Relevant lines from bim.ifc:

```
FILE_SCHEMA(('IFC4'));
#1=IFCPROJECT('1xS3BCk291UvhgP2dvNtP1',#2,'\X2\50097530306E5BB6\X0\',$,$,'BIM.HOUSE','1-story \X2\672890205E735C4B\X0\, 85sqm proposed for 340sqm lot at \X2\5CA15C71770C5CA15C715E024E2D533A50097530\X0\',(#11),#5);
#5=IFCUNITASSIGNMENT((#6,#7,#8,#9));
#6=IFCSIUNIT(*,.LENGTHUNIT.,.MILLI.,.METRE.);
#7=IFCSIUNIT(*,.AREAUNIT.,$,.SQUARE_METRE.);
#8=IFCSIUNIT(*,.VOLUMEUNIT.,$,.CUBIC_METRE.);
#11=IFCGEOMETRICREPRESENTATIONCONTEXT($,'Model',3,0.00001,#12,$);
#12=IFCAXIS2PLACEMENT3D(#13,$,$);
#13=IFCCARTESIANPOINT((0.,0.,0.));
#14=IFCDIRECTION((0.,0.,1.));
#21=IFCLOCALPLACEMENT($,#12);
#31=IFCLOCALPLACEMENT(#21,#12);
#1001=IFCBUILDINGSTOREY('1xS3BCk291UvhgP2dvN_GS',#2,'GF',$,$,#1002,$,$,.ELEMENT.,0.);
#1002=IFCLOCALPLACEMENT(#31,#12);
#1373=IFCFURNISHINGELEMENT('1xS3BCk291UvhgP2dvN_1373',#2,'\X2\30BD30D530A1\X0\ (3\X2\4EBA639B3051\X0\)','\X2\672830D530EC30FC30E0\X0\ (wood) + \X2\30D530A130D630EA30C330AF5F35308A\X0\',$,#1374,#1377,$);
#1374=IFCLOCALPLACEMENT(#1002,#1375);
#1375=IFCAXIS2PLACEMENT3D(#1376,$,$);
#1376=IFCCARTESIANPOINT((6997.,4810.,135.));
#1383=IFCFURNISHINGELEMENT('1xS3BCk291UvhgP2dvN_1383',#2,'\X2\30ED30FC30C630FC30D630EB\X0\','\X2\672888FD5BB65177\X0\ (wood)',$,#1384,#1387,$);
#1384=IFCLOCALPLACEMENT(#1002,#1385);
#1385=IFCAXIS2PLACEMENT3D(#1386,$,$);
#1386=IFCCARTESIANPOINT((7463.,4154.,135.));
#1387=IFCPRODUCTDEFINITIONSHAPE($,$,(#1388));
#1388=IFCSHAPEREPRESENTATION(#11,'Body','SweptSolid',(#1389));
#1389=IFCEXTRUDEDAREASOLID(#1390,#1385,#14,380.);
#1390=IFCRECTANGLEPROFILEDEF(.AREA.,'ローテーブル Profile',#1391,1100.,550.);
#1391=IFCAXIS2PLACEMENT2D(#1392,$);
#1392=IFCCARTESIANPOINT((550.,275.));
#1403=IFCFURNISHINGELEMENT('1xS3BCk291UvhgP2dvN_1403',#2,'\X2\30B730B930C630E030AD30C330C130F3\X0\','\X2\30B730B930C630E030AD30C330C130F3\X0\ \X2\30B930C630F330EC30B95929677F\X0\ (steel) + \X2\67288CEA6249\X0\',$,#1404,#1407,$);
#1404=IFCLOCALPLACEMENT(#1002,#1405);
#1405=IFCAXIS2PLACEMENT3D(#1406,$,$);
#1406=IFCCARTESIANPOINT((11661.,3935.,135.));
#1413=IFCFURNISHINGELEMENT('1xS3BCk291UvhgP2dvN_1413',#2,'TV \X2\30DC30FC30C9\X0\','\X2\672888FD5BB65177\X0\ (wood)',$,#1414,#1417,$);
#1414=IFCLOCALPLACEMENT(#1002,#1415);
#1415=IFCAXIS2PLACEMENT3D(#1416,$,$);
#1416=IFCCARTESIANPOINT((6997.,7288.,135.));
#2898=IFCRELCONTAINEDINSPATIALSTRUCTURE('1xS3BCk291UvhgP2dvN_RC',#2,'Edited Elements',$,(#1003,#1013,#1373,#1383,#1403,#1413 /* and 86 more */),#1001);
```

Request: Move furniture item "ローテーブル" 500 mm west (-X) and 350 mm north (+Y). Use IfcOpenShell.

```python
import ifcopenshell
import ifcopenshell.api.geometry
import ifcopenshell.util.placement
import ifcopenshell.util.unit

model = ifcopenshell.open("bim.ifc")
unit_scale = ifcopenshell.util.unit.calculate_unit_scale(model)

item = model.by_id(1383)
matrix = ifcopenshell.util.placement.get_local_placement(item.ObjectPlacement)
matrix[0, 3] -= 0.5 / unit_scale
matrix[1, 3] += 0.35 / unit_scale
ifcopenshell.api.geometry.edit_object_placement(model, product=item, matrix=matrix, is_si=False)

print(ifcopenshell.util.placement.get_local_placement(item.ObjectPlacement).round(3) + 0.0)

model.write("bim_v2.ifc")
```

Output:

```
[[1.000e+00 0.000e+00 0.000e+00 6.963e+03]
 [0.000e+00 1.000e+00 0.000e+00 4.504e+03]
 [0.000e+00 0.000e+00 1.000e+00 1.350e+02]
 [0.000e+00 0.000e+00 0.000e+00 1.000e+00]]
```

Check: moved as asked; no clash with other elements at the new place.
